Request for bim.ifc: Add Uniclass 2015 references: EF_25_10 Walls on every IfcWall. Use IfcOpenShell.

First a look at what the model holds.

```python
import ifcopenshell

model = ifcopenshell.open("bim.ifc")
print(model.schema)
print("classifications:", [c.Name for c in model.by_type("IfcClassification")])
for ifc_class in ("IfcDoor", "IfcRoof", "IfcStair", "IfcWall", "IfcWindow"):
    print(ifc_class, len(model.by_type(ifc_class)))
```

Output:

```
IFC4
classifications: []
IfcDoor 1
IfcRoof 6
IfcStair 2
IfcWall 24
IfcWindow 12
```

```python
import ifcopenshell
import ifcopenshell.api.classification

model = ifcopenshell.open("bim.ifc")

system = ifcopenshell.api.classification.add_classification(model, classification="Uniclass 2015")

codes = {
    "IfcWall": ("EF_25_10", "Walls"),
}
for ifc_class, (code, name) in codes.items():
    products = model.by_type(ifc_class)
    ifcopenshell.api.classification.add_reference(
        model, products=products, classification=system, identification=code, name=name
    )
    print(code, len(products))

model.write("bim-out.ifc")
```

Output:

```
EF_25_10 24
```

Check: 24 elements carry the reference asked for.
